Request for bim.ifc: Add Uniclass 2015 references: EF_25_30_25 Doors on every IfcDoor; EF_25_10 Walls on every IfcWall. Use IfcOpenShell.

First a look at what the model holds.

```python
import ifcopenshell

model = ifcopenshell.open("bim.ifc")
print(model.schema)
print("classifications:", [c.Name for c in model.by_type("IfcClassification")])
for ifc_class in ("IfcDoor", "IfcRoof", "IfcStair", "IfcWall", "IfcWindow"):
    print(ifc_class, len(model.by_type(ifc_class)))
```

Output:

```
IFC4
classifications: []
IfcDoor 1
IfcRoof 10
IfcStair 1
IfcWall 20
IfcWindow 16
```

```python
import ifcopenshell
import ifcopenshell.api.classification

model = ifcopenshell.open("bim.ifc")

system = ifcopenshell.api.classification.add_classification(model, classification="Uniclass 2015")

codes = {
    "IfcDoor": ("EF_25_30_25", "Doors"),
    "IfcWall": ("EF_25_10", "Walls"),
}
for ifc_class, (code, name) in codes.items():
    products = model.by_type(ifc_class)
    ifcopenshell.api.classification.add_reference(
        model, products=products, classification=system, identification=code, name=name
    )
    print(code, len(products))

model.write("bim_edited.ifc")
```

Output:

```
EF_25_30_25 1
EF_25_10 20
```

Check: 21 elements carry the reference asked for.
